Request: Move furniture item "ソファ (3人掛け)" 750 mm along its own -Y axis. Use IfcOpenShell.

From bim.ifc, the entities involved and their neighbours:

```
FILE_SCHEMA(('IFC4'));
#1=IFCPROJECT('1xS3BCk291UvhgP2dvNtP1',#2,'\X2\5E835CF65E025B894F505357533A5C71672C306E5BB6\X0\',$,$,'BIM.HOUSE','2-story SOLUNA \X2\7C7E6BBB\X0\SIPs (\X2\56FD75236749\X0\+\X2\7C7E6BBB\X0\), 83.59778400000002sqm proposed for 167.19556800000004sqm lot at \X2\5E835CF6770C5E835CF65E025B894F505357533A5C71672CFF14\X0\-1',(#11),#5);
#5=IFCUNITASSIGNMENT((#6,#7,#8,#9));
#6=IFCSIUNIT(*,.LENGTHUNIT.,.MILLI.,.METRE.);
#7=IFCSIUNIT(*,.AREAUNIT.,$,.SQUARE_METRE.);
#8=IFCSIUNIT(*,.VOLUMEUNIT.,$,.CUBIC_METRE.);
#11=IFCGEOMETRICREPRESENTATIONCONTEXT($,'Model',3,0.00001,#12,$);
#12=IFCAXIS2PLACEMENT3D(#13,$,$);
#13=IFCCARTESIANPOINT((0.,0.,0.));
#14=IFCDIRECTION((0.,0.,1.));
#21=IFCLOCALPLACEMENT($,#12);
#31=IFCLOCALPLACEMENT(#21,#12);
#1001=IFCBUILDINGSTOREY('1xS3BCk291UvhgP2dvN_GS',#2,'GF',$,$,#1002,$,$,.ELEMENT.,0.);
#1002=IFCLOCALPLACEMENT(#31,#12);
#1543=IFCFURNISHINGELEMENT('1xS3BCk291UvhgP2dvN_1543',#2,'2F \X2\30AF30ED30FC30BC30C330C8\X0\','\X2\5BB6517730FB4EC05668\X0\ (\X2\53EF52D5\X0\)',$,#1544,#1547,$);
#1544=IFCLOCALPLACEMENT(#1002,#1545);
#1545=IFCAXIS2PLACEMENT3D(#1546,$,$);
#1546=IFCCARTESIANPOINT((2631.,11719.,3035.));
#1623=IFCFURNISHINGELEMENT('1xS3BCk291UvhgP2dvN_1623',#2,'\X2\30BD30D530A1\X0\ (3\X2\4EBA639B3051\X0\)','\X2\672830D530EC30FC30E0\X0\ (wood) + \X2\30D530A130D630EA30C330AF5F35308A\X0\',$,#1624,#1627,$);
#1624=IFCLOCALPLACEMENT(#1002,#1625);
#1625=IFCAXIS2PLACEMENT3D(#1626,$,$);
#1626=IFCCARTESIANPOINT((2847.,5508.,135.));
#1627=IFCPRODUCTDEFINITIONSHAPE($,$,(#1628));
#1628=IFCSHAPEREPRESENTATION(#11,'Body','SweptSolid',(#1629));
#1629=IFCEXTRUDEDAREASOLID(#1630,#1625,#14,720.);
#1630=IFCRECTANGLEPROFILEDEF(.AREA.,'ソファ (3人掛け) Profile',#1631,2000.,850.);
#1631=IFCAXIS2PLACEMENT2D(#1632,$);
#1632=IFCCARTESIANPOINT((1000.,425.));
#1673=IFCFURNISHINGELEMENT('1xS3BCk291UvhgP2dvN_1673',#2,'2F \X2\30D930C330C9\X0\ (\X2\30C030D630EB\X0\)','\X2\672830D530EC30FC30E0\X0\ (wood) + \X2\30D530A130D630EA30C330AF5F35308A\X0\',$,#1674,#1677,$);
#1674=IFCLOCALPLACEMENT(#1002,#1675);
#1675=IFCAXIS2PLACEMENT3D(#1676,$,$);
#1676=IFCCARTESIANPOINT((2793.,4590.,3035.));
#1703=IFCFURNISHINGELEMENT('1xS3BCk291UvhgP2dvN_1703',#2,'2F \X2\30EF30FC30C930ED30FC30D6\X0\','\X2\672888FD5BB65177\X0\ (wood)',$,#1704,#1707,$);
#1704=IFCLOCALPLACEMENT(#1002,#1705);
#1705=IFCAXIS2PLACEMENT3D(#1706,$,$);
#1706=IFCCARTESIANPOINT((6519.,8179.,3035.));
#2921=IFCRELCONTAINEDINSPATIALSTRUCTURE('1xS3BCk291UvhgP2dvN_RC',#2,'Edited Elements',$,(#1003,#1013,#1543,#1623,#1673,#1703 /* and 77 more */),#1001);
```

```python
import ifcopenshell
import ifcopenshell.api.geometry
import ifcopenshell.util.placement

model = ifcopenshell.open("bim.ifc")

item = model.by_guid("1xS3BCk291UvhgP2dvN_1623")
matrix = ifcopenshell.util.placement.get_local_placement(item.ObjectPlacement)
matrix[:3, 3] -= matrix[:3, 1] * 750.0
ifcopenshell.api.geometry.edit_object_placement(model, product=item, matrix=matrix, is_si=False)

print(ifcopenshell.util.placement.get_local_placement(item.ObjectPlacement).round(3) + 0.0)

model.write("bim_edited.ifc")
```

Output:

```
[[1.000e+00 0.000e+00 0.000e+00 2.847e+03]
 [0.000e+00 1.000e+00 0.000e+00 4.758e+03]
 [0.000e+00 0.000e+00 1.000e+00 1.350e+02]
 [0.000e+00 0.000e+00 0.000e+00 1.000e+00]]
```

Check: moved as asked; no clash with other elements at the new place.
